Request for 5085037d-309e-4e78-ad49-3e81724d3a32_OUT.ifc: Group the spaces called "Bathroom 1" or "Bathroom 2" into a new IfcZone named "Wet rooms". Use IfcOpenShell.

First a look at what the model holds.

```python
import ifcopenshell

model = ifcopenshell.open("5085037d-309e-4e78-ad49-3e81724d3a32_OUT.ifc")
print(model.schema)
seen = {}
for space in model.by_type("IfcSpace"):
    seen[space.LongName] = seen.get(space.LongName, 0) + 1
for name, count in sorted(seen.items(), key=str):
    print(count, "x", name)
print("zones:", [z.Name for z in model.by_type("IfcZone")][:20])
```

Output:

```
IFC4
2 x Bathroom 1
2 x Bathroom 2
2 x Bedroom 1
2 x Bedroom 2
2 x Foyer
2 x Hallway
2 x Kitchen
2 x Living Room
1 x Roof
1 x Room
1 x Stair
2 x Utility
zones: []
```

```python
import ifcopenshell
import ifcopenshell.api.group
import ifcopenshell.api.root

model = ifcopenshell.open("5085037d-309e-4e78-ad49-3e81724d3a32_OUT.ifc")

names = {"Bathroom 1", "Bathroom 2"}
spaces = [s for s in model.by_type("IfcSpace") if s.LongName in names]

zone = ifcopenshell.api.root.create_entity(model, ifc_class="IfcZone", name="Wet rooms")
ifcopenshell.api.group.assign_group(model, products=spaces, group=zone)
print(len(spaces), "spaces in", zone.Name)

model.write("5085037d-309e-4e78-ad49-3e81724d3a32_OUT-out.ifc")
```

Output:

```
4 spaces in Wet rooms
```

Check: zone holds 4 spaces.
